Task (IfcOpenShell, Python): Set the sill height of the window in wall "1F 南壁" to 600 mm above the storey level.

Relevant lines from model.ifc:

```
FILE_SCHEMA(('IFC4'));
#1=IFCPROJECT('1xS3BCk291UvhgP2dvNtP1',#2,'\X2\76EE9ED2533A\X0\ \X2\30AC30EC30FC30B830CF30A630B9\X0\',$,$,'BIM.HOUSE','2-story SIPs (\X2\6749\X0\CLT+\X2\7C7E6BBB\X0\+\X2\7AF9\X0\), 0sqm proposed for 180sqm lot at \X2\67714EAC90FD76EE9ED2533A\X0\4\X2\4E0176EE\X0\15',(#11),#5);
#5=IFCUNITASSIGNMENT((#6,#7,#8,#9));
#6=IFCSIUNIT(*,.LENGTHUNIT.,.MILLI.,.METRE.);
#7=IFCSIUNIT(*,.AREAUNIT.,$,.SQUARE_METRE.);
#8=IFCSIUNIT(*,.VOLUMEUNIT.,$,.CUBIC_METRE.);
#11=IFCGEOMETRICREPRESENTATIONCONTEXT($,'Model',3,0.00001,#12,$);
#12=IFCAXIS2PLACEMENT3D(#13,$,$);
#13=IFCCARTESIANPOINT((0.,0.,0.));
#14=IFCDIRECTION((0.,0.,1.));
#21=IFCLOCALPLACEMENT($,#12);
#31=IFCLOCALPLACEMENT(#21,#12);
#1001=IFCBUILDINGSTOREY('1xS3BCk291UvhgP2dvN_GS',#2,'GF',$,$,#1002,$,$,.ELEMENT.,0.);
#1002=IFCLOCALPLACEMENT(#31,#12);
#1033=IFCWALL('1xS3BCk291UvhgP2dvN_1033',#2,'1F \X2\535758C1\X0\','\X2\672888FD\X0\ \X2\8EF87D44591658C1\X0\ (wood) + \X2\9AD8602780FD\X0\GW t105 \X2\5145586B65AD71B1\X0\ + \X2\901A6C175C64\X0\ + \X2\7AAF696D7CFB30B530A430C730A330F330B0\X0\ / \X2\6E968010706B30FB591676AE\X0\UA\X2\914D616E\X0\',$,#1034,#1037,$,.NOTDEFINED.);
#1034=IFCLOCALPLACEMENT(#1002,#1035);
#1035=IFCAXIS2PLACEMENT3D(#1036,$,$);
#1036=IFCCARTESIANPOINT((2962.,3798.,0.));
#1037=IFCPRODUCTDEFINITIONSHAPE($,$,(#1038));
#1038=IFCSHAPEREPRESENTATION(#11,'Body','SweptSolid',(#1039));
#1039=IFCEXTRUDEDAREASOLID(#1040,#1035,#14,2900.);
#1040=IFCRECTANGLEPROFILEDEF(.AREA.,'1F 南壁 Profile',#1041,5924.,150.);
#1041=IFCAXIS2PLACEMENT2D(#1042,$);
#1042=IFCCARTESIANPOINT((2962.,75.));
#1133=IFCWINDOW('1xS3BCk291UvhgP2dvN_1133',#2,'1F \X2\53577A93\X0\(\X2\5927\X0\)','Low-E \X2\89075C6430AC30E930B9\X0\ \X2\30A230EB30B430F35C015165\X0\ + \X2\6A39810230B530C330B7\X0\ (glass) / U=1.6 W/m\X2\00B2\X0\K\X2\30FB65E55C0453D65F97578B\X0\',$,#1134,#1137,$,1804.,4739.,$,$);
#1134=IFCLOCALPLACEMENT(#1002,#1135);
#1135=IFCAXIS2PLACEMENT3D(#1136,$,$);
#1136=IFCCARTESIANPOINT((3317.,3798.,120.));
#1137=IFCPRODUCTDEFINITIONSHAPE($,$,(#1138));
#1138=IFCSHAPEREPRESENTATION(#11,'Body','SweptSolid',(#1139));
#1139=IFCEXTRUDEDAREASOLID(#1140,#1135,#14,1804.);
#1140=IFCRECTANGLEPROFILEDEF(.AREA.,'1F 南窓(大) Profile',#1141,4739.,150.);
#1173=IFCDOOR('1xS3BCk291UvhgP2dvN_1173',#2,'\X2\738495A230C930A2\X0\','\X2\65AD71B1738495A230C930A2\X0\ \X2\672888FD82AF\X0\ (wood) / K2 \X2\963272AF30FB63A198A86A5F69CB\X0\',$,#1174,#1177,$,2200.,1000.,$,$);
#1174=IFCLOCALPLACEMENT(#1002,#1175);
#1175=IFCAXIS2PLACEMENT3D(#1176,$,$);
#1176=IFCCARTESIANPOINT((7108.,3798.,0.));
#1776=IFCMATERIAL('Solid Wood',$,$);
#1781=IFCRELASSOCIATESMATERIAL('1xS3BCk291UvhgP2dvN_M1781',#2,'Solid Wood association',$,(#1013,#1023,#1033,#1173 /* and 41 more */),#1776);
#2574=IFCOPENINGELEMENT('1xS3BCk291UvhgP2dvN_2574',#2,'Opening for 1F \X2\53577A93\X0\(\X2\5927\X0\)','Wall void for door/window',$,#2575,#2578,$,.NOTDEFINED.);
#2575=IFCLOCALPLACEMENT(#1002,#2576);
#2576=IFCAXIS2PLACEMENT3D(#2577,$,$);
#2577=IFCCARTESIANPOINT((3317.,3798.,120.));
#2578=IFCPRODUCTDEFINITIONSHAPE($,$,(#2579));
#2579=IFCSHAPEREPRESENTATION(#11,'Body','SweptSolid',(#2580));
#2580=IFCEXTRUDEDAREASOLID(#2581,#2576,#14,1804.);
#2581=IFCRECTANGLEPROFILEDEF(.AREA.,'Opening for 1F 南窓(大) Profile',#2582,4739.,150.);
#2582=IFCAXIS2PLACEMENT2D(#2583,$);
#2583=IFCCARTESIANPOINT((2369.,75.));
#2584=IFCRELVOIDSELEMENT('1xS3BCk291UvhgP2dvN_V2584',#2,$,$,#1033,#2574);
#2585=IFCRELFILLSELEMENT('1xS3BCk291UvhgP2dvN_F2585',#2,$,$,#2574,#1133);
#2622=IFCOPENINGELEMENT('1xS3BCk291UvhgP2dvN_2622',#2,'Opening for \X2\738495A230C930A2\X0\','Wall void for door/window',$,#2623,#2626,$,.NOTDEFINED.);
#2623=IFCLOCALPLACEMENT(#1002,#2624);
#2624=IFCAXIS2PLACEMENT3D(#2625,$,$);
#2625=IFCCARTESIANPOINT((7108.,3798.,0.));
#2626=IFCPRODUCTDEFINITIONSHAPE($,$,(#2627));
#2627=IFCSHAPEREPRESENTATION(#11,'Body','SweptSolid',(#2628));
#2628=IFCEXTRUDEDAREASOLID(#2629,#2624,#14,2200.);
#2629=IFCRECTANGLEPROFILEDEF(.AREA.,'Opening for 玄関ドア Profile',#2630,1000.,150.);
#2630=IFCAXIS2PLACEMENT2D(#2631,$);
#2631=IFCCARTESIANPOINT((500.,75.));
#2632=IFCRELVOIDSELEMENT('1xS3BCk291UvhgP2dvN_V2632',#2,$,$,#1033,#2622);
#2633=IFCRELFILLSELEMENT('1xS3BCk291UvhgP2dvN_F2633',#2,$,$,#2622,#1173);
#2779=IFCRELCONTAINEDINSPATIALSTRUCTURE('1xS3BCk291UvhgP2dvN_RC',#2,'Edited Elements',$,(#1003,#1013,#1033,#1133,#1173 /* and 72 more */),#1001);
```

```python
import numpy as np
import ifcopenshell
import ifcopenshell.api.geometry
import ifcopenshell.geom
import ifcopenshell.util.element
import ifcopenshell.util.placement
import ifcopenshell.util.shape
import ifcopenshell.util.unit

model = ifcopenshell.open("model.ifc")
unit_scale = ifcopenshell.util.unit.calculate_unit_scale(model)

window = model.by_id(1133)
opening = window.FillsVoids[0].RelatingOpeningElement
storey = ifcopenshell.util.element.get_container(window, ifc_class="IfcBuildingStorey")
level = ifcopenshell.util.placement.get_local_placement(storey.ObjectPlacement)[2, 3]

# The opening's origin need not be at the sill, so measure its lowest point.
shape = ifcopenshell.geom.create_shape(ifcopenshell.geom.settings(), opening)
bottom = ifcopenshell.util.shape.get_shape_bottom_elevation(shape, shape.geometry) / unit_scale
dz = level + 0.6 / unit_scale - bottom

shift = np.array([0.0, 0.0, dz])
# The window is not placed relative to its opening, so move both.
for product in (opening, window):
    matrix = ifcopenshell.util.placement.get_local_placement(product.ObjectPlacement)
    matrix[:3, 3] += shift
    ifcopenshell.api.geometry.edit_object_placement(model, product=product, matrix=matrix, is_si=False)

print(f"moved by {dz * unit_scale:+.3f} m")

model.write("model_rev.ifc")
```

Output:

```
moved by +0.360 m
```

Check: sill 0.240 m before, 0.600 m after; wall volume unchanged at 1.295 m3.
